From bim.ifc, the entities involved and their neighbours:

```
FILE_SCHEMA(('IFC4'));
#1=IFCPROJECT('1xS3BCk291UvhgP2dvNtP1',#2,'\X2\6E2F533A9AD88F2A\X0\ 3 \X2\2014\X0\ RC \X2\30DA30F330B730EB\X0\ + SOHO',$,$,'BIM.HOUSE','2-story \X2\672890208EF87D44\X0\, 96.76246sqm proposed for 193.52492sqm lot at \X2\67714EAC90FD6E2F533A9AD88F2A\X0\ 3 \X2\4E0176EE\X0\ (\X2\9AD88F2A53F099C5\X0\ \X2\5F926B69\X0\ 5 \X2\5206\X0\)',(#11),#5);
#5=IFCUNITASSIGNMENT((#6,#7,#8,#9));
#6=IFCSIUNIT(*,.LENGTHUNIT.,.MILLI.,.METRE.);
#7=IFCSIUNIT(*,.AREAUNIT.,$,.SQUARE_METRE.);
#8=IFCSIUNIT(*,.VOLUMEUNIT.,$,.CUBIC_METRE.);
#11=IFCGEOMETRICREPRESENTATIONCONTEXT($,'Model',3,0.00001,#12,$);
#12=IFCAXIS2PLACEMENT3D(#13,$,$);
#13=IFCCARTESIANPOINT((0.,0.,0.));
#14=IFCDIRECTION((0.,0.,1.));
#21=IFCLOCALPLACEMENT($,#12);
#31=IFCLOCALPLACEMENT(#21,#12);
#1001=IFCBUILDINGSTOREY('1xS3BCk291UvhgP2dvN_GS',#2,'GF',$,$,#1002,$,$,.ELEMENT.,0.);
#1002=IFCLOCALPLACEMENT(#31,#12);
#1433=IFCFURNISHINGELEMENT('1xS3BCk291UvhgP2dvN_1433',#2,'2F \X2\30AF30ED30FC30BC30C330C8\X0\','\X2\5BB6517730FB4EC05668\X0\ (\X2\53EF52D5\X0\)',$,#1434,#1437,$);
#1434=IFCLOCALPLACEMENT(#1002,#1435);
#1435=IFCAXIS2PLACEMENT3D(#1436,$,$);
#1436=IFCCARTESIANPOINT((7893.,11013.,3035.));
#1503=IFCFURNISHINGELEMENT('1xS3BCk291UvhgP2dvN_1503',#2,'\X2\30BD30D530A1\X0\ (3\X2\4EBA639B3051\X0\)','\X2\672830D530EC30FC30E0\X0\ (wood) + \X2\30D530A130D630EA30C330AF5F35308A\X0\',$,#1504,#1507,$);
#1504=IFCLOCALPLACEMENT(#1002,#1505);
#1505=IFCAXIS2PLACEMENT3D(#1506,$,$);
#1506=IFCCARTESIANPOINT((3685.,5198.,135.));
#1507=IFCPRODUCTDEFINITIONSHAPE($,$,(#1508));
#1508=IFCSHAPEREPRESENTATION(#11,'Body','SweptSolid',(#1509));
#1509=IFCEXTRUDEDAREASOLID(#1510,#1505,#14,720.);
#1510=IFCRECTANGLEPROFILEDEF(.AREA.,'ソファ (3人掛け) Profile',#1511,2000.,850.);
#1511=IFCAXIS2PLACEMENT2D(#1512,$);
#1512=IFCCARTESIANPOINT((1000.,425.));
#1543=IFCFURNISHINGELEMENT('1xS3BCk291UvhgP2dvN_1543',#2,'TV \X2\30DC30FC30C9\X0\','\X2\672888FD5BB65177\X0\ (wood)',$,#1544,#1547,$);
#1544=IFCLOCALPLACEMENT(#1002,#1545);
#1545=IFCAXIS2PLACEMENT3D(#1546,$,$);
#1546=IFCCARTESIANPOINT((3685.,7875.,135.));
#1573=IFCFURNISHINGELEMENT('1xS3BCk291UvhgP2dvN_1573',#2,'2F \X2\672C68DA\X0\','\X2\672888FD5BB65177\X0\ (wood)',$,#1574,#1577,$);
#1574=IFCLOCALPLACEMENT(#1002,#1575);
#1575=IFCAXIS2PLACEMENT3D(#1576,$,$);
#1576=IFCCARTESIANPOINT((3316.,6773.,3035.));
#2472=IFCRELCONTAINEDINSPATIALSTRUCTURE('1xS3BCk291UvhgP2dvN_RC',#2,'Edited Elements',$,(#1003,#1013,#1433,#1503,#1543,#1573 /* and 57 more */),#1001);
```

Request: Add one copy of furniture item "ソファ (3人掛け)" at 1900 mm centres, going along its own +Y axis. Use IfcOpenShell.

```python
import ifcopenshell
import ifcopenshell.api.geometry
import ifcopenshell.api.root
import ifcopenshell.util.element
import ifcopenshell.util.placement
import ifcopenshell.util.unit

model = ifcopenshell.open("bim.ifc")
unit_scale = ifcopenshell.util.unit.calculate_unit_scale(model)


def reuse_history(source, copy):
    """copy_class also copies each property set's owner history, people and application; keep the originals."""
    for rel in copy.IsDefinedBy:
        if rel.is_a("IfcRelDefinesByProperties") and (history := rel.RelatingPropertyDefinition.OwnerHistory):
            rel.RelatingPropertyDefinition.OwnerHistory = source.OwnerHistory
            ifcopenshell.util.element.remove_deep2(model, history)


source = model.by_guid("1xS3BCk291UvhgP2dvN_1503")
base = ifcopenshell.util.placement.get_local_placement(source.ObjectPlacement)
step = base[:3, 1] * 1.9 / unit_scale

for i in range(1, 2):
    copy = ifcopenshell.api.root.copy_class(model, product=source)
    copy.Representation = ifcopenshell.util.element.copy_deep(
        model, source.Representation, exclude=["IfcGeometricRepresentationContext", "IfcRepresentationMap"]
    )
    reuse_history(source, copy)
    matrix = base.copy()
    matrix[:3, 3] += i * step
    print("added at", matrix[:3, 3].round(3) + 0.0)
    ifcopenshell.api.geometry.edit_object_placement(model, product=copy, matrix=matrix, is_si=False)

model.write("bim_v2.ifc")
```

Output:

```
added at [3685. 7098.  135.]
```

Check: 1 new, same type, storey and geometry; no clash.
